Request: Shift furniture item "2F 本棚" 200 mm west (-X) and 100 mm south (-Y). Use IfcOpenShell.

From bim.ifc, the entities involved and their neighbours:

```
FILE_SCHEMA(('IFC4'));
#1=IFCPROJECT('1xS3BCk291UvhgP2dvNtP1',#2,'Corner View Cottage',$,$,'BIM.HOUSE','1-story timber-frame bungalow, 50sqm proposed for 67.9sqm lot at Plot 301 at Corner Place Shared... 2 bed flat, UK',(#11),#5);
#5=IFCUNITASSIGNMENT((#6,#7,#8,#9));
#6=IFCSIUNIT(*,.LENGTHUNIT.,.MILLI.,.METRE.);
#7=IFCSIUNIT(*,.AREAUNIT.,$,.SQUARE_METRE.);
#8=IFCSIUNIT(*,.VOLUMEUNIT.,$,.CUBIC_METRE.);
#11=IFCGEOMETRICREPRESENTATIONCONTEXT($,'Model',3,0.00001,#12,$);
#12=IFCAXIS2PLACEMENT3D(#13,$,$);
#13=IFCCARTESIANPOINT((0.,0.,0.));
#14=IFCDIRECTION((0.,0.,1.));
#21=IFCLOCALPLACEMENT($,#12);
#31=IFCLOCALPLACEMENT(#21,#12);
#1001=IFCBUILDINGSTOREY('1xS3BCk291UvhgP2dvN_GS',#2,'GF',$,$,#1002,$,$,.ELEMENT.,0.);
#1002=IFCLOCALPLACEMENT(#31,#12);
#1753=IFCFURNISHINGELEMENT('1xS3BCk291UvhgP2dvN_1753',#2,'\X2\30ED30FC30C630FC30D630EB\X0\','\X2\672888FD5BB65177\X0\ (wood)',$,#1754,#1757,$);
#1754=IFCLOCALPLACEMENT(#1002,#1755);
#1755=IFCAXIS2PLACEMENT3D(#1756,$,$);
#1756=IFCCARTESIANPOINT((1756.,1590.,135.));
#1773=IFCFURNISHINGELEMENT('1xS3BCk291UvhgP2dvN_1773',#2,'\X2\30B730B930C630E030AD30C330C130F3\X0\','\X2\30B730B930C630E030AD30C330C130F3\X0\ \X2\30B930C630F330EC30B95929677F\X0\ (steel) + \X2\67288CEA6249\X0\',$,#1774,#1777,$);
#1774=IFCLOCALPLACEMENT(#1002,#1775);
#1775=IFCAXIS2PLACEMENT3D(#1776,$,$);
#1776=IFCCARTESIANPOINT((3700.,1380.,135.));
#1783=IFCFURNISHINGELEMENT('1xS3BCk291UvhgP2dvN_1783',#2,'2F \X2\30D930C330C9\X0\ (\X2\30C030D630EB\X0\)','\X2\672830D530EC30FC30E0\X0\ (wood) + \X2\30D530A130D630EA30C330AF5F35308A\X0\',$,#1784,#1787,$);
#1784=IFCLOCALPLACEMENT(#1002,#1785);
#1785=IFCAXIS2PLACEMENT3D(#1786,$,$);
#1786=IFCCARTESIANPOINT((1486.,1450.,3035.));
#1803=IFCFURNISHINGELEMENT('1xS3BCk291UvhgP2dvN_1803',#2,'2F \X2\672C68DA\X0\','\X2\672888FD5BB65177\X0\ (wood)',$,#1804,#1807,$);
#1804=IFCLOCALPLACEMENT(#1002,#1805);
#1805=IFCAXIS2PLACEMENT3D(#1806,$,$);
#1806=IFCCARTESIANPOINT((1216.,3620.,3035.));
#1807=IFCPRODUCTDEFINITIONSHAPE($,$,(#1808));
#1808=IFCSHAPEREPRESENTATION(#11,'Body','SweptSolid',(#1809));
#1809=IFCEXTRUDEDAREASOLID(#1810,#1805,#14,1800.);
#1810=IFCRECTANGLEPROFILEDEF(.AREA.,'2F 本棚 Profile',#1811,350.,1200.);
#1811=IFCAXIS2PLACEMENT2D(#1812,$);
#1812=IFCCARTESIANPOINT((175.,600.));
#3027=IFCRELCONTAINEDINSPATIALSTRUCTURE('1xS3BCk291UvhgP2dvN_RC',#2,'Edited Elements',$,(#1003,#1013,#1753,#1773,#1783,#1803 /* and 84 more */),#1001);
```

```python
import ifcopenshell
import ifcopenshell.api.geometry
import ifcopenshell.util.placement
import ifcopenshell.util.unit

model = ifcopenshell.open("bim.ifc")
unit_scale = ifcopenshell.util.unit.calculate_unit_scale(model)

item = model.by_guid("1xS3BCk291UvhgP2dvN_1803")
matrix = ifcopenshell.util.placement.get_local_placement(item.ObjectPlacement)
matrix[0, 3] -= 0.2 / unit_scale
matrix[1, 3] -= 0.1 / unit_scale
ifcopenshell.api.geometry.edit_object_placement(model, product=item, matrix=matrix, is_si=False)

print(ifcopenshell.util.placement.get_local_placement(item.ObjectPlacement).round(3) + 0.0)

model.write("bim_v2.ifc")
```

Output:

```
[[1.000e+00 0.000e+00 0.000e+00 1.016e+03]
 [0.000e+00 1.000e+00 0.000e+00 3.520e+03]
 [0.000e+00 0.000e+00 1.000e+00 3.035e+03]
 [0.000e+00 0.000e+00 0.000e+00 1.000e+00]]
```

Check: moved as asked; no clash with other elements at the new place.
